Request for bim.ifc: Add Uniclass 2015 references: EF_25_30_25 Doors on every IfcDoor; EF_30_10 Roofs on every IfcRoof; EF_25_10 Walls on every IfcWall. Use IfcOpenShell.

First a look at what the model holds.

```python
import ifcopenshell

model = ifcopenshell.open("bim.ifc")
print(model.schema)
print("classifications:", [c.Name for c in model.by_type("IfcClassification")])
for ifc_class in ("IfcDoor", "IfcRoof", "IfcStair", "IfcWall", "IfcWindow"):
    print(ifc_class, len(model.by_type(ifc_class)))
```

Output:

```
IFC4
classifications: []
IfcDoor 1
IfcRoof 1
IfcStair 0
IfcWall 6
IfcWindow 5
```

```python
import ifcopenshell
import ifcopenshell.api.classification

model = ifcopenshell.open("bim.ifc")

system = ifcopenshell.api.classification.add_classification(model, classification="Uniclass 2015")

codes = {
    "IfcDoor": ("EF_25_30_25", "Doors"),
    "IfcRoof": ("EF_30_10", "Roofs"),
    "IfcWall": ("EF_25_10", "Walls"),
}
for ifc_class, (code, name) in codes.items():
    products = model.by_type(ifc_class)
    ifcopenshell.api.classification.add_reference(
        model, products=products, classification=system, identification=code, name=name
    )
    print(code, len(products))

model.write("bim_rev.ifc")
```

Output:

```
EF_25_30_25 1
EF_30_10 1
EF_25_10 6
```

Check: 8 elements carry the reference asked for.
